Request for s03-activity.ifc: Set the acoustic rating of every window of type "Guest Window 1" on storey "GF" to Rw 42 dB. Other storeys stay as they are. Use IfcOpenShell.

First a look at what the model holds.

```python
import ifcopenshell
import ifcopenshell.util.element

model = ifcopenshell.open("s03-activity.ifc")
print(model.schema)
storey = next(s for s in model.by_type("IfcBuildingStorey") if s.Name == "GF")
windows = [e for e in ifcopenshell.util.element.get_decomposition(storey) if e.is_a("IfcWindow")]
seen = {}
for e in windows:
    element_type = ifcopenshell.util.element.get_type(e)
    key = (element_type.Name if element_type != e and element_type else None, ifcopenshell.util.element.get_pset(e, "Pset_WindowCommon", "AcousticRating"))
    seen[key] = seen.get(key, 0) + 1
for (name, value), count in sorted(seen.items(), key=str):
    print(count, "x", name, "|", value)
```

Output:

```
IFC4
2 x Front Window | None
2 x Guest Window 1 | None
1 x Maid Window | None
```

```python
import ifcopenshell
import ifcopenshell.api.pset
import ifcopenshell.util.element

model = ifcopenshell.open("s03-activity.ifc")

storey = next(s for s in model.by_type("IfcBuildingStorey") if s.Name == "GF")
windows = [e for e in ifcopenshell.util.element.get_decomposition(storey) if e.is_a("IfcWindow")]

count = 0
for e in windows:
    element_type = ifcopenshell.util.element.get_type(e)
    if element_type in (None, e) or element_type.Name != "Guest Window 1":
        continue
    # add_pset returns the element's existing set when there is one.
    pset = ifcopenshell.api.pset.add_pset(model, product=e, name="Pset_WindowCommon")
    ifcopenshell.api.pset.edit_pset(model, pset=pset, properties={"AcousticRating": "Rw 42 dB"})
    count += 1

print(count, "windows updated")

model.write("s03-activity_edited.ifc")
```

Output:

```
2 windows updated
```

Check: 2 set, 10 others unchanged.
